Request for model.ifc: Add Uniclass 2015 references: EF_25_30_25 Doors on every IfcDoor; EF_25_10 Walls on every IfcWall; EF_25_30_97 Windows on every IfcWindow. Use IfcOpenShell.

First a look at what the model holds.

```python
import ifcopenshell

model = ifcopenshell.open("model.ifc")
print(model.schema)
print("classifications:", [c.Name for c in model.by_type("IfcClassification")])
for ifc_class in ("IfcDoor", "IfcRoof", "IfcStair", "IfcWall", "IfcWindow"):
    print(ifc_class, len(model.by_type(ifc_class)))
```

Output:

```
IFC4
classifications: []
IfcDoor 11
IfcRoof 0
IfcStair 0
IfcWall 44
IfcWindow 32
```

```python
import ifcopenshell
import ifcopenshell.api.classification

model = ifcopenshell.open("model.ifc")

system = ifcopenshell.api.classification.add_classification(model, classification="Uniclass 2015")

codes = {
    "IfcDoor": ("EF_25_30_25", "Doors"),
    "IfcWall": ("EF_25_10", "Walls"),
    "IfcWindow": ("EF_25_30_97", "Windows"),
}
for ifc_class, (code, name) in codes.items():
    products = model.by_type(ifc_class)
    ifcopenshell.api.classification.add_reference(
        model, products=products, classification=system, identification=code, name=name
    )
    print(code, len(products))

model.write("model-out.ifc")
```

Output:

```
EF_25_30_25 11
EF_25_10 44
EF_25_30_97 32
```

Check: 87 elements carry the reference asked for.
